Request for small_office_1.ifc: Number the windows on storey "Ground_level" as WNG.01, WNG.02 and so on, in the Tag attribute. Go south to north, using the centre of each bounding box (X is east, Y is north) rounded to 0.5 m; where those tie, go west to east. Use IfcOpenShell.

First a look at what the model holds.

```python
import ifcopenshell
import ifcopenshell.util.element
import ifcopenshell.util.placement

model = ifcopenshell.open("small_office_1.ifc")
print(model.schema)
storey = next(s for s in model.by_type("IfcBuildingStorey") if s.Name == "Ground_level")
windows = [e for e in ifcopenshell.util.element.get_decomposition(storey) if e.is_a("IfcWindow")]
for e in sorted(windows, key=lambda e: e.id()):
    origin = ifcopenshell.util.placement.get_local_placement(e.ObjectPlacement)[:3, 3]
    print(e.id(), e.Tag, e.Name, origin.round(2) + 0.0, sep=" | ")
```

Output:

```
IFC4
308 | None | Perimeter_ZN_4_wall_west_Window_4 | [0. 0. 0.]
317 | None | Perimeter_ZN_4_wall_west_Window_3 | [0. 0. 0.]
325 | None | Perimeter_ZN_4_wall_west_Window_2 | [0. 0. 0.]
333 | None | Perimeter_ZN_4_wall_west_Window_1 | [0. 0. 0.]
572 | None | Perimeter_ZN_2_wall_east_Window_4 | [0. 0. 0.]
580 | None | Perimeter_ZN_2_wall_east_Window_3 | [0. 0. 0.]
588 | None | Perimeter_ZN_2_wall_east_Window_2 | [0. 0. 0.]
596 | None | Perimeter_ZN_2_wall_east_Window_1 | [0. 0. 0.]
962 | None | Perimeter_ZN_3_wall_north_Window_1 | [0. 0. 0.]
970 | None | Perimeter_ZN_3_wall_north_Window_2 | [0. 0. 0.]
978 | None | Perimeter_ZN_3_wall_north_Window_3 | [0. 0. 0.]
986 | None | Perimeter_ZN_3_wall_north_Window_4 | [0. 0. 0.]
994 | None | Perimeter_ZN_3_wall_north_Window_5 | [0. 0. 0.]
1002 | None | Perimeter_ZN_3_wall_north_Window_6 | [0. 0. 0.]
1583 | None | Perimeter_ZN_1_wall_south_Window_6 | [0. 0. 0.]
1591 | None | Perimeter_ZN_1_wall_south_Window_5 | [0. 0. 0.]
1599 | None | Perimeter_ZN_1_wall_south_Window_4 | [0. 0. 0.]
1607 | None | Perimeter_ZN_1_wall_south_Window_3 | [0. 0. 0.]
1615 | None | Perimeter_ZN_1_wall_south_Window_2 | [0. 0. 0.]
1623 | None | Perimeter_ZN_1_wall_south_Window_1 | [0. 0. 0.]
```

```python
import ifcopenshell
import ifcopenshell.geom
import ifcopenshell.util.element
import ifcopenshell.util.shape

model = ifcopenshell.open("small_office_1.ifc")
settings = ifcopenshell.geom.settings()
settings.set("use-world-coords", True)


def centre(element):
    shape = ifcopenshell.geom.create_shape(settings, element)
    return ifcopenshell.util.shape.get_bbox_centroid(shape.geometry)


storey = next(s for s in model.by_type("IfcBuildingStorey") if s.Name == "Ground_level")
windows = [e for e in ifcopenshell.util.element.get_decomposition(storey) if e.is_a("IfcWindow")]

# Insertion points can sit at a corner or the storey origin, so sort by the geometry (in metres).
centres = {e: centre(e) for e in windows}
windows.sort(key=lambda e: (round(centres[e][1] / 0.5), centres[e][0]))

for i, e in enumerate(windows, start=1):
    number = f"WNG.{i:02d}"
    e.Tag = number
    print(e.id(), number)

model.write("small_office_1_edited.ifc")
```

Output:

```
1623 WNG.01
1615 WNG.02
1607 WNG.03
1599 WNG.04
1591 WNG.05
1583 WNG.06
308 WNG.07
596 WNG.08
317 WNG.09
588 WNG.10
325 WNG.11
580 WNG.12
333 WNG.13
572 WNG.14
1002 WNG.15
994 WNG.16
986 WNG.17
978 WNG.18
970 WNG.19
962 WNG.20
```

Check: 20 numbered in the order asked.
